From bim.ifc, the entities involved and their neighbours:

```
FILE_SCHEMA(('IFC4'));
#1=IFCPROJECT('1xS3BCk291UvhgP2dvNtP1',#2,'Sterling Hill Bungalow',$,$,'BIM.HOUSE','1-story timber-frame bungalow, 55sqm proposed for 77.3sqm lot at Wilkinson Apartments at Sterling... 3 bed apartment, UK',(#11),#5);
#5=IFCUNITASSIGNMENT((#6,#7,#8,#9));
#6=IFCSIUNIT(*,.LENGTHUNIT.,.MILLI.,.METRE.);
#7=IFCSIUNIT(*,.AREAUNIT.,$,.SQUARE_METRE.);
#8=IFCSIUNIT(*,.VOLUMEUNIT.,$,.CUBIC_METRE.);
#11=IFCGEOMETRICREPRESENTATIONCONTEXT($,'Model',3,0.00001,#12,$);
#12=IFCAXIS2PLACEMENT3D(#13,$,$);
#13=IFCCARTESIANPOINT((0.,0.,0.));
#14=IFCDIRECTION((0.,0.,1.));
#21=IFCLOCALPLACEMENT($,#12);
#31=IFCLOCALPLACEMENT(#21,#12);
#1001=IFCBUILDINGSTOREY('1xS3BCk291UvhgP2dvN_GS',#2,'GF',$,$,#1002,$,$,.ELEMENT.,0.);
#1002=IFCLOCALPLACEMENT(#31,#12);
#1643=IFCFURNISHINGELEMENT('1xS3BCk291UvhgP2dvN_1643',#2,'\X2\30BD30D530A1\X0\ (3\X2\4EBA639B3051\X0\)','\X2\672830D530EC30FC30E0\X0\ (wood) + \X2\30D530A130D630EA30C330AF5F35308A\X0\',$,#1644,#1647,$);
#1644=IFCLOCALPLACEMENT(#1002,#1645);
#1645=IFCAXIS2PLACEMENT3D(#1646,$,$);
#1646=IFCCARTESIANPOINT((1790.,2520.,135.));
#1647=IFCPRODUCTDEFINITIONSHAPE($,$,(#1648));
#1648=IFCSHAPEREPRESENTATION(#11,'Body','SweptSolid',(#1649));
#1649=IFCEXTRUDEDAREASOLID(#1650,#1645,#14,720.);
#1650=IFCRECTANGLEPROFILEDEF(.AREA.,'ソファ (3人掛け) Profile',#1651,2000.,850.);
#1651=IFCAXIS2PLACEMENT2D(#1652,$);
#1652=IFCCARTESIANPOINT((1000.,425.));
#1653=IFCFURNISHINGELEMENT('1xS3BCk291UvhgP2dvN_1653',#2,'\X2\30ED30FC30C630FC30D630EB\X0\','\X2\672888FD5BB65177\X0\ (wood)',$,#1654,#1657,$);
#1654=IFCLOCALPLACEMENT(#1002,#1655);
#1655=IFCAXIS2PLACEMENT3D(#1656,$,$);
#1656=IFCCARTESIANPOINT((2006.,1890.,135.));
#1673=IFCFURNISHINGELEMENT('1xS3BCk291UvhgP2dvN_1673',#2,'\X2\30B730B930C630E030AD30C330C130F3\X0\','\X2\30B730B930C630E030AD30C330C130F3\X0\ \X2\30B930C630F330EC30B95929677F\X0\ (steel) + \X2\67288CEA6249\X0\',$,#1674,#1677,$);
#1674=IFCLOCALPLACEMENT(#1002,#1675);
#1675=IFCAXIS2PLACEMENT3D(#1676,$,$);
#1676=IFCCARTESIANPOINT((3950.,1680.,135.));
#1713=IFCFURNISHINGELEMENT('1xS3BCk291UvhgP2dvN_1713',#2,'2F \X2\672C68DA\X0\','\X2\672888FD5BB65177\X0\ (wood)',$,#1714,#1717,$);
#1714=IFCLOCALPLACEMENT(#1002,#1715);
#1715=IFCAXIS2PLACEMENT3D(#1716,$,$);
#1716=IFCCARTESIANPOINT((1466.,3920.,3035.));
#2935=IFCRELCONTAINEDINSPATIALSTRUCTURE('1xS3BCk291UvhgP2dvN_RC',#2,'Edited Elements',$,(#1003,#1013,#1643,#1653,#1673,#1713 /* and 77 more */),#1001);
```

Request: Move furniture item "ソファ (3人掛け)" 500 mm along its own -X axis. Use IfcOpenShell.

```python
import ifcopenshell
import ifcopenshell.api.geometry
import ifcopenshell.util.placement
import ifcopenshell.util.unit

model = ifcopenshell.open("bim.ifc")
unit_scale = ifcopenshell.util.unit.calculate_unit_scale(model)

item = model.by_id(1643)
matrix = ifcopenshell.util.placement.get_local_placement(item.ObjectPlacement)
matrix[:3, 3] -= matrix[:3, 0] * 0.5 / unit_scale
ifcopenshell.api.geometry.edit_object_placement(model, product=item, matrix=matrix, is_si=False)

print(ifcopenshell.util.placement.get_local_placement(item.ObjectPlacement).round(3) + 0.0)

model.write("bim_rev.ifc")
```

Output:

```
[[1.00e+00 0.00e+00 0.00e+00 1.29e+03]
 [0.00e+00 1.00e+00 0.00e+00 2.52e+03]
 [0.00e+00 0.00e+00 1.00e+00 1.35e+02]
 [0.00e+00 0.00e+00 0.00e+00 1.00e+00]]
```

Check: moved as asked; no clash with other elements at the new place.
